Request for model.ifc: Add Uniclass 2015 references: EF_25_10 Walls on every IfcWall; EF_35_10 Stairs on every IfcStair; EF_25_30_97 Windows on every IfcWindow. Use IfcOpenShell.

First a look at what the model holds.

```python
import ifcopenshell

model = ifcopenshell.open("model.ifc")
print(model.schema)
print("classifications:", [c.Name for c in model.by_type("IfcClassification")])
for ifc_class in ("IfcDoor", "IfcRoof", "IfcStair", "IfcWall", "IfcWindow"):
    print(ifc_class, len(model.by_type(ifc_class)))
```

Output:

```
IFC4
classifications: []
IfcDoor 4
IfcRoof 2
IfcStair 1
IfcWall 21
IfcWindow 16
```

```python
import ifcopenshell
import ifcopenshell.api.classification

model = ifcopenshell.open("model.ifc")

system = ifcopenshell.api.classification.add_classification(model, classification="Uniclass 2015")

codes = {
    "IfcWall": ("EF_25_10", "Walls"),
    "IfcStair": ("EF_35_10", "Stairs"),
    "IfcWindow": ("EF_25_30_97", "Windows"),
}
for ifc_class, (code, name) in codes.items():
    products = model.by_type(ifc_class)
    ifcopenshell.api.classification.add_reference(
        model, products=products, classification=system, identification=code, name=name
    )
    print(code, len(products))

model.write("model_v2.ifc")
```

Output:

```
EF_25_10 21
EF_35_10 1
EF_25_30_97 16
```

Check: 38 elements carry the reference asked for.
